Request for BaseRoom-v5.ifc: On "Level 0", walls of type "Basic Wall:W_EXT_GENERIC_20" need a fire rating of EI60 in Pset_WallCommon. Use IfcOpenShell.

First a look at what the model holds.

```python
import ifcopenshell
import ifcopenshell.util.element

model = ifcopenshell.open("BaseRoom-v5.ifc")
print(model.schema)
storey = next(s for s in model.by_type("IfcBuildingStorey") if s.Name == "Level 0")
walls = [e for e in ifcopenshell.util.element.get_decomposition(storey) if e.is_a("IfcWall")]
seen = {}
for e in walls:
    element_type = ifcopenshell.util.element.get_type(e)
    key = (element_type.Name if element_type != e and element_type else None, ifcopenshell.util.element.get_pset(e, "Pset_WallCommon", "FireRating"))
    seen[key] = seen.get(key, 0) + 1
for (name, value), count in sorted(seen.items(), key=str):
    print(count, "x", name, "|", value)
```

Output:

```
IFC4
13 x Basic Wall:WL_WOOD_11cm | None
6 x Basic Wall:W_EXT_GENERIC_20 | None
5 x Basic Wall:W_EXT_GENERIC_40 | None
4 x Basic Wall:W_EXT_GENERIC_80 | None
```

```python
import ifcopenshell
import ifcopenshell.api.pset
import ifcopenshell.util.element

model = ifcopenshell.open("BaseRoom-v5.ifc")

storey = next(s for s in model.by_type("IfcBuildingStorey") if s.Name == "Level 0")
walls = [e for e in ifcopenshell.util.element.get_decomposition(storey) if e.is_a("IfcWall")]

count = 0
for e in walls:
    element_type = ifcopenshell.util.element.get_type(e)
    if element_type in (None, e) or element_type.Name != "Basic Wall:W_EXT_GENERIC_20":
        continue
    # add_pset returns the element's existing set when there is one.
    pset = ifcopenshell.api.pset.add_pset(model, product=e, name="Pset_WallCommon")
    ifcopenshell.api.pset.edit_pset(model, pset=pset, properties={"FireRating": "EI60"})
    count += 1

print(count, "walls updated")

model.write("BaseRoom-v5_v2.ifc")
```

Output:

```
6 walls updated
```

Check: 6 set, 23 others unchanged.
